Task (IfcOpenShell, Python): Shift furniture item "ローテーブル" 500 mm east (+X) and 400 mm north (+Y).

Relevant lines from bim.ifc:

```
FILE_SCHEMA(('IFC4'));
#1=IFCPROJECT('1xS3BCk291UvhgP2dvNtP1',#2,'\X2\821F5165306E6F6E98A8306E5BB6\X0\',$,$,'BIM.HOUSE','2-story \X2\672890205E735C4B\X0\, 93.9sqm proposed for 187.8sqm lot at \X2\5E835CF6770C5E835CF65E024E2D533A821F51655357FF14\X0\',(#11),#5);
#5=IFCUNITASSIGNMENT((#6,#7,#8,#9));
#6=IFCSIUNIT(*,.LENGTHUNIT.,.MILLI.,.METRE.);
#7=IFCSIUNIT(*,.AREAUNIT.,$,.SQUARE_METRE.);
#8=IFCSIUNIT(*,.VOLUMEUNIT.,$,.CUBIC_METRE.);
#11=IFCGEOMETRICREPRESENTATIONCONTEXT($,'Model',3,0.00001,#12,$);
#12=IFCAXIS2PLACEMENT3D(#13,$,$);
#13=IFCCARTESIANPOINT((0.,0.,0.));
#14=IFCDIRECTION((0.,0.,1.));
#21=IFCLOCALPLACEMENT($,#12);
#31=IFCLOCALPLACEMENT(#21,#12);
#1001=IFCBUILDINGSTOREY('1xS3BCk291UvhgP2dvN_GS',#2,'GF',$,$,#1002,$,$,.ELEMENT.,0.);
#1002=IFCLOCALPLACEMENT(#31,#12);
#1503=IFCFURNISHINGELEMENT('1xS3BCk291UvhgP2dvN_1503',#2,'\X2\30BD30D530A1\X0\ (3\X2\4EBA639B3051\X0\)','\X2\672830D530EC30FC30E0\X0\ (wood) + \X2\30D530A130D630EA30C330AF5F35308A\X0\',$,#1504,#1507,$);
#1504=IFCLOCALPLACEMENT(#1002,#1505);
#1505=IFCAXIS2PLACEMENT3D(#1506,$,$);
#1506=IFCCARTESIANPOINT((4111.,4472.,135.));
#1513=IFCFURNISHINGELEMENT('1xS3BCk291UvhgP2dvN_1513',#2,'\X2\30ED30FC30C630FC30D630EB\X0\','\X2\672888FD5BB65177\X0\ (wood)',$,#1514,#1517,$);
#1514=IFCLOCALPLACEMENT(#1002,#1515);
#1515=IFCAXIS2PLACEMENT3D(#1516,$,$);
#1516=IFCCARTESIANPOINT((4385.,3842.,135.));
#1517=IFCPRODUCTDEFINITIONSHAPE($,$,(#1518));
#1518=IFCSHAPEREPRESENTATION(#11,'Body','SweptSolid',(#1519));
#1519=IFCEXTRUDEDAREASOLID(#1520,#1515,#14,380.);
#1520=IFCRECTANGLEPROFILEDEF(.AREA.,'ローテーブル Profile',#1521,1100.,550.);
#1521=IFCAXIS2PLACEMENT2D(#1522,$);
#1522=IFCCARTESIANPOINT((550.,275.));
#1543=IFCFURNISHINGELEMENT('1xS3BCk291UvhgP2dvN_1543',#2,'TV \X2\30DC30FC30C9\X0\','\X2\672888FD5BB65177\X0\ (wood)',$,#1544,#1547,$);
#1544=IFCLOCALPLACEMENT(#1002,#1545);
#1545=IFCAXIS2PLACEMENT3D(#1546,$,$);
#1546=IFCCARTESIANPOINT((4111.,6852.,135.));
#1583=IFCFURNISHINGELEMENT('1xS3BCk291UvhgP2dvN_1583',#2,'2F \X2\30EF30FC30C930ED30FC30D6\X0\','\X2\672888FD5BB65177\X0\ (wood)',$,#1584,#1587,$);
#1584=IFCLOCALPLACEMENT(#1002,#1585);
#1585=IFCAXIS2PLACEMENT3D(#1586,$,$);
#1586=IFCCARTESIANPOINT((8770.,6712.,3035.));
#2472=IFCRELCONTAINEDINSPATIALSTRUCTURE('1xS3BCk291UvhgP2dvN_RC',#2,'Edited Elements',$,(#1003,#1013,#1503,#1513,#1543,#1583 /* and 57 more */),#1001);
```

```python
import ifcopenshell
import ifcopenshell.api.geometry
import ifcopenshell.util.placement

model = ifcopenshell.open("bim.ifc")

item = model.by_guid("1xS3BCk291UvhgP2dvN_1513")
matrix = ifcopenshell.util.placement.get_local_placement(item.ObjectPlacement)
matrix[0, 3] += 500.0
matrix[1, 3] += 400.0
ifcopenshell.api.geometry.edit_object_placement(model, product=item, matrix=matrix, is_si=False)

print(ifcopenshell.util.placement.get_local_placement(item.ObjectPlacement).round(3) + 0.0)

model.write("bim-out.ifc")
```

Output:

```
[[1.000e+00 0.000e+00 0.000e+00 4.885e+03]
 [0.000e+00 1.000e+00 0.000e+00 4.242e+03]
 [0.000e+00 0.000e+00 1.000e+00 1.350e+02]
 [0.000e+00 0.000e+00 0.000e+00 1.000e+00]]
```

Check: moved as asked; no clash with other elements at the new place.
